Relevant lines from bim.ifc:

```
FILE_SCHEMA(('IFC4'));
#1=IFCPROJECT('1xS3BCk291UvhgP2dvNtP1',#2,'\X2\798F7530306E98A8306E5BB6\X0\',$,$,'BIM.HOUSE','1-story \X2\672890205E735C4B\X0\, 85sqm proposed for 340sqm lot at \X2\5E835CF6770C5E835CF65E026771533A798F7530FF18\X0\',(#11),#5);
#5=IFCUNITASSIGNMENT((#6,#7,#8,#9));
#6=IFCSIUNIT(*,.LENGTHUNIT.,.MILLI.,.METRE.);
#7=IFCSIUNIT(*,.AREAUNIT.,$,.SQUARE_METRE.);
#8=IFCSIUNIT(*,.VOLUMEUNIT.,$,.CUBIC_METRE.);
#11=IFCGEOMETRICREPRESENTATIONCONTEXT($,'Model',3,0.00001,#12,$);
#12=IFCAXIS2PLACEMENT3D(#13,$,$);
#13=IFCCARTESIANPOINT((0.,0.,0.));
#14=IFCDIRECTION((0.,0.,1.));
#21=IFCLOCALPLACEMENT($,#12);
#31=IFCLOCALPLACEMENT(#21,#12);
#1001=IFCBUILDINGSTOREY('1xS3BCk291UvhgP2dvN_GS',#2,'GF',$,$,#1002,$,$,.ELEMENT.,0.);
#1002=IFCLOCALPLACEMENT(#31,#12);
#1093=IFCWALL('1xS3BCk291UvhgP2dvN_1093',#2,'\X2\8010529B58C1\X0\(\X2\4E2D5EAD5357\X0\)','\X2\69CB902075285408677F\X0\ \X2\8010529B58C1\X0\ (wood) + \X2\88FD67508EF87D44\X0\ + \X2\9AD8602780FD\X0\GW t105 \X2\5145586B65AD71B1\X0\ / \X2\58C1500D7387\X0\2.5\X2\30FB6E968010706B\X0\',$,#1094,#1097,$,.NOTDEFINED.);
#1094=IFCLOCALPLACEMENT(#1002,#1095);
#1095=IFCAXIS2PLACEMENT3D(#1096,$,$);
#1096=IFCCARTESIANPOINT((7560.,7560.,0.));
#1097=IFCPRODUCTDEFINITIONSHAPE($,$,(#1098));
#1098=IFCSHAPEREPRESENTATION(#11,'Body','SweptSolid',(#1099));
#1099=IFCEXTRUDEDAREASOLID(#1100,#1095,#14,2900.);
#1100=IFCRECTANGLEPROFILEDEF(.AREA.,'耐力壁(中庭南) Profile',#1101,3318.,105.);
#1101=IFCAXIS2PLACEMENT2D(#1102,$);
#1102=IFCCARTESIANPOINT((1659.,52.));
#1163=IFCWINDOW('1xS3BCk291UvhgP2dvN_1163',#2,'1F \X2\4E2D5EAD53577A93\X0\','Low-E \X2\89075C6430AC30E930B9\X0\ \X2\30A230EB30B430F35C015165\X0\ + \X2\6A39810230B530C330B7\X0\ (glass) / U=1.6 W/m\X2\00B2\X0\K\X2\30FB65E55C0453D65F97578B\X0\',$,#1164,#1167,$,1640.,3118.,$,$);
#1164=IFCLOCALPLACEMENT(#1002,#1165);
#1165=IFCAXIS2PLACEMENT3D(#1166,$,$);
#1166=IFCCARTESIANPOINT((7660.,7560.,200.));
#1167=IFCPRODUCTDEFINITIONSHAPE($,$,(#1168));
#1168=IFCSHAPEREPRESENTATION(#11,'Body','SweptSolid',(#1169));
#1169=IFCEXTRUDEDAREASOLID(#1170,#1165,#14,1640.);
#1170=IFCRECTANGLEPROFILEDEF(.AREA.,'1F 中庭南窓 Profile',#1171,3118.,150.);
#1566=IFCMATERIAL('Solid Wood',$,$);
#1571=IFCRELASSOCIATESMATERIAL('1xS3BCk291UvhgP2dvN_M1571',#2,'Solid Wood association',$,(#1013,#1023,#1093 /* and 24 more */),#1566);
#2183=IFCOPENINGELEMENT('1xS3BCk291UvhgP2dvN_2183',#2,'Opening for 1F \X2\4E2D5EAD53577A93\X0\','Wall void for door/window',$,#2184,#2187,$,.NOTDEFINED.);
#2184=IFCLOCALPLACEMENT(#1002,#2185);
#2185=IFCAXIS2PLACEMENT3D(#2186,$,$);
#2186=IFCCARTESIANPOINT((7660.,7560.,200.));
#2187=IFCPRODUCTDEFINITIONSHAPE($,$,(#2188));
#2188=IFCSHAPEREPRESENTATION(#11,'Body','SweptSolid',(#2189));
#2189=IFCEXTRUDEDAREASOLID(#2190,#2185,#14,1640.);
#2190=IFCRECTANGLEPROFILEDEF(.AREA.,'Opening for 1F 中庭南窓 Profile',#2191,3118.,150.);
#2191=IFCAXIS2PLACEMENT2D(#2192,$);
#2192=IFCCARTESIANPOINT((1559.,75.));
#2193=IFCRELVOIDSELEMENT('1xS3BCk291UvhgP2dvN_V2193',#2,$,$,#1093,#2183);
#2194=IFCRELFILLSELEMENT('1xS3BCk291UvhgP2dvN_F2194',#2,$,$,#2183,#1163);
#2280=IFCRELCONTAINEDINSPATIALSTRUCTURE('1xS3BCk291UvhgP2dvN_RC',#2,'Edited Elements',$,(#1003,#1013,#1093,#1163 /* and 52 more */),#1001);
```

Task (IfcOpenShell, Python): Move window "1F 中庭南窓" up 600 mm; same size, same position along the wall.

```python
import numpy as np
import ifcopenshell
import ifcopenshell.api.geometry
import ifcopenshell.util.placement
import ifcopenshell.util.unit

model = ifcopenshell.open("bim.ifc")
unit_scale = ifcopenshell.util.unit.calculate_unit_scale(model)

window = model.by_guid("1xS3BCk291UvhgP2dvN_1163")
opening = window.FillsVoids[0].RelatingOpeningElement
dz = 0.6 / unit_scale

shift = np.array([0.0, 0.0, dz])
# The window is not placed relative to its opening, so move both.
for product in (opening, window):
    matrix = ifcopenshell.util.placement.get_local_placement(product.ObjectPlacement)
    matrix[:3, 3] += shift
    ifcopenshell.api.geometry.edit_object_placement(model, product=product, matrix=matrix, is_si=False)

print(f"moved by {dz * unit_scale:+.3f} m")

model.write("bim-out.ifc")
```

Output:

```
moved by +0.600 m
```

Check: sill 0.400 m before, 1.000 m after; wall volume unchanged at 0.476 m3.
